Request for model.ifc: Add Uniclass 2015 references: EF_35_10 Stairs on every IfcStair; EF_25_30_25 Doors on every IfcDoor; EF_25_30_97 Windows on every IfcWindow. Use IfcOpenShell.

First a look at what the model holds.

```python
import ifcopenshell

model = ifcopenshell.open("model.ifc")
print(model.schema)
print("classifications:", [c.Name for c in model.by_type("IfcClassification")])
for ifc_class in ("IfcDoor", "IfcRoof", "IfcStair", "IfcWall", "IfcWindow"):
    print(ifc_class, len(model.by_type(ifc_class)))
```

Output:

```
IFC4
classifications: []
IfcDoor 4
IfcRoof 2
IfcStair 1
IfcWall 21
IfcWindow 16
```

```python
import ifcopenshell
import ifcopenshell.api.classification

model = ifcopenshell.open("model.ifc")

system = ifcopenshell.api.classification.add_classification(model, classification="Uniclass 2015")

codes = {
    "IfcStair": ("EF_35_10", "Stairs"),
    "IfcDoor": ("EF_25_30_25", "Doors"),
    "IfcWindow": ("EF_25_30_97", "Windows"),
}
for ifc_class, (code, name) in codes.items():
    products = model.by_type(ifc_class)
    ifcopenshell.api.classification.add_reference(
        model, products=products, classification=system, identification=code, name=name
    )
    print(code, len(products))

model.write("model_rev.ifc")
```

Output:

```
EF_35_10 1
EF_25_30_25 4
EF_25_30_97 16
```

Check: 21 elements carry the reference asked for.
